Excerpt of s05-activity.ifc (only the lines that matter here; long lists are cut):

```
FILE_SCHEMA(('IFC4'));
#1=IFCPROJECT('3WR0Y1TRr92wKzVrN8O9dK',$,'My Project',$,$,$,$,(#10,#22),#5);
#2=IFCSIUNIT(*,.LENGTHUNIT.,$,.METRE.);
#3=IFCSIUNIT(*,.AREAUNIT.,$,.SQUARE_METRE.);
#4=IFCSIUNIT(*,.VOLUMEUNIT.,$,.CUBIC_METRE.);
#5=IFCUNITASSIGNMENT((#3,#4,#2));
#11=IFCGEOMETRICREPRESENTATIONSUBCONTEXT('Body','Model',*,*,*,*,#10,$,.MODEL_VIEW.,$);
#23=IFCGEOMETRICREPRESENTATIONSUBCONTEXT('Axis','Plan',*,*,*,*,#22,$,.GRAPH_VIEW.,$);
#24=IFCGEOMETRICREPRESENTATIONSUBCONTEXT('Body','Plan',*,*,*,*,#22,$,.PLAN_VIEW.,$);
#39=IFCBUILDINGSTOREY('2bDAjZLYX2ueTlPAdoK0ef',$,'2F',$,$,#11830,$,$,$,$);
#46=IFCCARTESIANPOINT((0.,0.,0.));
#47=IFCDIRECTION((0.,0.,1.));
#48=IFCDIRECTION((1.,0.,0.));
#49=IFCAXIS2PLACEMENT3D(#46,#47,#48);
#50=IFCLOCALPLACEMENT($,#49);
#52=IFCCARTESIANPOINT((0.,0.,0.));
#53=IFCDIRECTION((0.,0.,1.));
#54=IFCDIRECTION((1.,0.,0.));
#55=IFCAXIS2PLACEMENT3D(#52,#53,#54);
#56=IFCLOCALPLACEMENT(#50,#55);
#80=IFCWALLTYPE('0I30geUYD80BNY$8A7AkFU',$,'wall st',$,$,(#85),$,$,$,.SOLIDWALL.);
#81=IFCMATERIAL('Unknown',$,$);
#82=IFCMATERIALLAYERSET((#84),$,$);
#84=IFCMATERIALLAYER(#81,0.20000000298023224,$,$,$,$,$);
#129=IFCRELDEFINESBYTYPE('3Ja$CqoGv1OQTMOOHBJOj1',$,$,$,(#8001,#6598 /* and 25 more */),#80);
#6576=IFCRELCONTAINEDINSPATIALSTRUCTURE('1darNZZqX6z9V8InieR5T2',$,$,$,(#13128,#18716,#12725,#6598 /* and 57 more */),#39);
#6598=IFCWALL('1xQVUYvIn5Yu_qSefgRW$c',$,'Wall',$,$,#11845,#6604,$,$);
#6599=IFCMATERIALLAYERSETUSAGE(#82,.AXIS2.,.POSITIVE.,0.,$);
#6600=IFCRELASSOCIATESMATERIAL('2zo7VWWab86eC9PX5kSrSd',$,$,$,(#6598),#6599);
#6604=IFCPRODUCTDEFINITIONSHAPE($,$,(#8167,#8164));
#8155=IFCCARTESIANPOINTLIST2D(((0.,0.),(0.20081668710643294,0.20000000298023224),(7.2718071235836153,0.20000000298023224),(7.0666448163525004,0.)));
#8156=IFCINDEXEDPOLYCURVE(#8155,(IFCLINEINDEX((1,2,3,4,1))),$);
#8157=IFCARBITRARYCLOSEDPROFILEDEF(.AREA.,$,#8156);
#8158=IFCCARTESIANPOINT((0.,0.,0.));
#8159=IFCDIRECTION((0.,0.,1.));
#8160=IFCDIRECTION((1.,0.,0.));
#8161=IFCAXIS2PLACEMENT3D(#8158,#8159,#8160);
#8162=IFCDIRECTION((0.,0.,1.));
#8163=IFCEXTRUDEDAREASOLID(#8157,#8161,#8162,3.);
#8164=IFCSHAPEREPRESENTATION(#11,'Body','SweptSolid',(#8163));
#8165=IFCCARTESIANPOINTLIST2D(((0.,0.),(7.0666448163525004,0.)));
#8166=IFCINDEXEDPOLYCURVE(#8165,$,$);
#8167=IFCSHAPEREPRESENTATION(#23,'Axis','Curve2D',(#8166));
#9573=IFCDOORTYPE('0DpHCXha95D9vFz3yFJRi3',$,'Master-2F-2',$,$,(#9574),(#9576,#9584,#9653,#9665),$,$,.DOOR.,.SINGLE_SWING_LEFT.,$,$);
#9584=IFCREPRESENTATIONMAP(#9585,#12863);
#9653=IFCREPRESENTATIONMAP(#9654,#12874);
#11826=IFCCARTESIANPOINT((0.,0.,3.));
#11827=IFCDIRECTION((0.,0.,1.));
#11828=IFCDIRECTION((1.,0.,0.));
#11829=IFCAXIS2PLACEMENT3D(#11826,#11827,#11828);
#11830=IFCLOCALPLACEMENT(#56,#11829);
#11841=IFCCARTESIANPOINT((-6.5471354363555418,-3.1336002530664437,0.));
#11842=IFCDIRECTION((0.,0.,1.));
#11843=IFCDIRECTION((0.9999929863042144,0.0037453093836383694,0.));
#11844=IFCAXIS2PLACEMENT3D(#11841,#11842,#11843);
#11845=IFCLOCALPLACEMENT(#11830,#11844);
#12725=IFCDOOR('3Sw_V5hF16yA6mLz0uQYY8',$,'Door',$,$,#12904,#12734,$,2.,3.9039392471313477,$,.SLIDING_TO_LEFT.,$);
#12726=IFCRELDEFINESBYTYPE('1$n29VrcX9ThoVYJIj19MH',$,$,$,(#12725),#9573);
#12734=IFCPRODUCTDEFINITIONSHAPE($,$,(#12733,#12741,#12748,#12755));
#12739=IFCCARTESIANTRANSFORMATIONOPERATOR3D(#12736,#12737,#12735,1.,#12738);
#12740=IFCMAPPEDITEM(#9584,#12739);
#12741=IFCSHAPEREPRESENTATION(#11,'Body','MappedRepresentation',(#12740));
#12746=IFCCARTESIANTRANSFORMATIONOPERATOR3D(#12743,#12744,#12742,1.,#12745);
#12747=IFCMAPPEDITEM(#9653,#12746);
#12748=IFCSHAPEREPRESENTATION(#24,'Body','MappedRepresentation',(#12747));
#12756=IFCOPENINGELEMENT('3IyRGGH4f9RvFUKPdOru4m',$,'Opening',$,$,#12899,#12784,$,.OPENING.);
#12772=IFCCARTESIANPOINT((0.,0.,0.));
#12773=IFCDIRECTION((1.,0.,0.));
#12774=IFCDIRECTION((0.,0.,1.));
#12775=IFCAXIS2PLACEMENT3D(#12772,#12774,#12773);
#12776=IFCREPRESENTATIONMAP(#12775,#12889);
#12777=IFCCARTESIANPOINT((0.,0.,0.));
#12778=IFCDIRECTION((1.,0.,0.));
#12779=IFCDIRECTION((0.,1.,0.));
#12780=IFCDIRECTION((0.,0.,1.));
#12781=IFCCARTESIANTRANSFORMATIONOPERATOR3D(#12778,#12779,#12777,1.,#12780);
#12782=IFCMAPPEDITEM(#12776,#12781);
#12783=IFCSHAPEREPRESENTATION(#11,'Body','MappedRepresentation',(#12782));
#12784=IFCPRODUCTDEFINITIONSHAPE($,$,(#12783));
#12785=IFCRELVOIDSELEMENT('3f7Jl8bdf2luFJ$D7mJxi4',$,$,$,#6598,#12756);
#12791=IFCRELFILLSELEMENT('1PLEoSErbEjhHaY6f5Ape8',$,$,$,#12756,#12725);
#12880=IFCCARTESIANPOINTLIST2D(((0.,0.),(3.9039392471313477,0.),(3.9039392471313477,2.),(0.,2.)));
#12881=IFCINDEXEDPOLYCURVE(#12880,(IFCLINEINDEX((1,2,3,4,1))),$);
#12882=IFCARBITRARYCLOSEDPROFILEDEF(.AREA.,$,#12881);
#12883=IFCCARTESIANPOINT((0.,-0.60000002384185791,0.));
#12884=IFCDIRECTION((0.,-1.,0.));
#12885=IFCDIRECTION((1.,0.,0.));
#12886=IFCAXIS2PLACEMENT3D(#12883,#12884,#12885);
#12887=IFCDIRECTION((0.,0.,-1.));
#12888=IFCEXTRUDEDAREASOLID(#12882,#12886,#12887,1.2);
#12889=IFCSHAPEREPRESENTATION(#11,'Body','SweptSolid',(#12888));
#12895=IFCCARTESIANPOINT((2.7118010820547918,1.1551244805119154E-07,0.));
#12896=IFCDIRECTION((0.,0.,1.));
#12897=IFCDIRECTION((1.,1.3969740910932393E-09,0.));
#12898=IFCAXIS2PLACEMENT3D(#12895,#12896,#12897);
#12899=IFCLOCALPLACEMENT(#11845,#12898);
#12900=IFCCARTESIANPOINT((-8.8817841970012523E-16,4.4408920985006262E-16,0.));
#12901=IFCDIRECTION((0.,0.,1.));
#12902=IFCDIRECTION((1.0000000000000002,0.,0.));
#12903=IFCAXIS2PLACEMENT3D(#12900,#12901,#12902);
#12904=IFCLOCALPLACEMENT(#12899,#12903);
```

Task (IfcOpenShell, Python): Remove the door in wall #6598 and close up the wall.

```python
import ifcopenshell
import ifcopenshell.api.feature
import ifcopenshell.api.root
import ifcopenshell.geom
import ifcopenshell.util.shape

model = ifcopenshell.open("s05-activity.ifc")
settings = ifcopenshell.geom.settings()


def volume(element):
    """Net volume in cubic metres, openings subtracted."""
    shape = ifcopenshell.geom.create_shape(settings, element)
    return ifcopenshell.util.shape.get_volume(shape.geometry)


door = model.by_id(12725)
opening = door.FillsVoids[0].RelatingOpeningElement
wall = opening.VoidsElements[0].RelatingBuildingElement
before = volume(wall)

ifcopenshell.api.root.remove_product(model, product=door)
ifcopenshell.api.feature.remove_feature(model, feature=opening)

after = volume(wall)

print(f"wall volume {before:.3f} -> {after:.3f} m3")

model.write("s05-activity_updated.ifc")
```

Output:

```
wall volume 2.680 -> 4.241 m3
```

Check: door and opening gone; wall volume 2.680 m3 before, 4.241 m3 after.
